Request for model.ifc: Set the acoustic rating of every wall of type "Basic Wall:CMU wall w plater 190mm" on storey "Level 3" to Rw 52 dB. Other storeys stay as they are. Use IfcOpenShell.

First a look at what the model holds.

```python
import ifcopenshell
import ifcopenshell.util.element

model = ifcopenshell.open("model.ifc")
print(model.schema)
storey = next(s for s in model.by_type("IfcBuildingStorey") if s.Name == "Level 3")
walls = [e for e in ifcopenshell.util.element.get_decomposition(storey) if e.is_a("IfcWall")]
seen = {}
for e in walls:
    element_type = ifcopenshell.util.element.get_type(e)
    key = (element_type.Name if element_type != e and element_type else None, ifcopenshell.util.element.get_pset(e, "Pset_WallCommon", "AcousticRating"))
    seen[key] = seen.get(key, 0) + 1
for (name, value), count in sorted(seen.items(), key=str):
    print(count, "x", name, "|", value)
```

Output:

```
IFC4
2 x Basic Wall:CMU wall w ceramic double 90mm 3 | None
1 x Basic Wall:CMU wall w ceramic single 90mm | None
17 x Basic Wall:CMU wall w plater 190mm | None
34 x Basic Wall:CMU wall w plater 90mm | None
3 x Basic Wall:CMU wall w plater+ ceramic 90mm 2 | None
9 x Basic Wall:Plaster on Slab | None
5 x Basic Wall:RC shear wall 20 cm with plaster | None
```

```python
import ifcopenshell
import ifcopenshell.api.pset
import ifcopenshell.util.element

model = ifcopenshell.open("model.ifc")

storey = next(s for s in model.by_type("IfcBuildingStorey") if s.Name == "Level 3")
walls = [e for e in ifcopenshell.util.element.get_decomposition(storey) if e.is_a("IfcWall")]

count = 0
for e in walls:
    element_type = ifcopenshell.util.element.get_type(e)
    if element_type in (None, e) or element_type.Name != "Basic Wall:CMU wall w plater 190mm":
        continue
    # add_pset returns the element's existing set when there is one.
    pset = ifcopenshell.api.pset.add_pset(model, product=e, name="Pset_WallCommon")
    ifcopenshell.api.pset.edit_pset(model, pset=pset, properties={"AcousticRating": "Rw 52 dB"})
    count += 1

print(count, "walls updated")

model.write("model_rev.ifc")
```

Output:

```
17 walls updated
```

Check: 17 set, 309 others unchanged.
